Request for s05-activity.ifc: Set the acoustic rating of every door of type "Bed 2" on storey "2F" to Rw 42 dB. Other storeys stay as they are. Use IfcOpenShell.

First a look at what the model holds.

```python
import ifcopenshell
import ifcopenshell.util.element

model = ifcopenshell.open("s05-activity.ifc")
print(model.schema)
storey = next(s for s in model.by_type("IfcBuildingStorey") if s.Name == "2F")
doors = [e for e in ifcopenshell.util.element.get_decomposition(storey) if e.is_a("IfcDoor")]
seen = {}
for e in doors:
    element_type = ifcopenshell.util.element.get_type(e)
    key = (element_type.Name if element_type != e and element_type else None, ifcopenshell.util.element.get_pset(e, "Pset_DoorCommon", "AcousticRating"))
    seen[key] = seen.get(key, 0) + 1
for (name, value), count in sorted(seen.items(), key=str):
    print(count, "x", name, "|", value)
```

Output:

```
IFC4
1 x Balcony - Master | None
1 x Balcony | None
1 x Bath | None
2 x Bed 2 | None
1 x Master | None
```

```python
import ifcopenshell
import ifcopenshell.api.pset
import ifcopenshell.util.element

model = ifcopenshell.open("s05-activity.ifc")

storey = next(s for s in model.by_type("IfcBuildingStorey") if s.Name == "2F")
doors = [e for e in ifcopenshell.util.element.get_decomposition(storey) if e.is_a("IfcDoor")]

count = 0
for e in doors:
    element_type = ifcopenshell.util.element.get_type(e)
    if element_type in (None, e) or element_type.Name != "Bed 2":
        continue
    # add_pset returns the element's existing set when there is one.
    pset = ifcopenshell.api.pset.add_pset(model, product=e, name="Pset_DoorCommon")
    ifcopenshell.api.pset.edit_pset(model, pset=pset, properties={"AcousticRating": "Rw 42 dB"})
    count += 1

print(count, "doors updated")

model.write("s05-activity_edited.ifc")
```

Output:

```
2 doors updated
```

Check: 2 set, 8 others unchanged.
